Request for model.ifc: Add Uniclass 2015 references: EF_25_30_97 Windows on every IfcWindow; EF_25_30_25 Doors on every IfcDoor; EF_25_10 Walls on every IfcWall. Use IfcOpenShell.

First a look at what the model holds.

```python
import ifcopenshell

model = ifcopenshell.open("model.ifc")
print(model.schema)
print("classifications:", [c.Name for c in model.by_type("IfcClassification")])
for ifc_class in ("IfcDoor", "IfcRoof", "IfcStair", "IfcWall", "IfcWindow"):
    print(ifc_class, len(model.by_type(ifc_class)))
```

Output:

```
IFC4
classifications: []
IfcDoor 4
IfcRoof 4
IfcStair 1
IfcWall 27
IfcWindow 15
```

```python
import ifcopenshell
import ifcopenshell.api.classification

model = ifcopenshell.open("model.ifc")

system = ifcopenshell.api.classification.add_classification(model, classification="Uniclass 2015")

codes = {
    "IfcWindow": ("EF_25_30_97", "Windows"),
    "IfcDoor": ("EF_25_30_25", "Doors"),
    "IfcWall": ("EF_25_10", "Walls"),
}
for ifc_class, (code, name) in codes.items():
    products = model.by_type(ifc_class)
    ifcopenshell.api.classification.add_reference(
        model, products=products, classification=system, identification=code, name=name
    )
    print(code, len(products))

model.write("model_edited.ifc")
```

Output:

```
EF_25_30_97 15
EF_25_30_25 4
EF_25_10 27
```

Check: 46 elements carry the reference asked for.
